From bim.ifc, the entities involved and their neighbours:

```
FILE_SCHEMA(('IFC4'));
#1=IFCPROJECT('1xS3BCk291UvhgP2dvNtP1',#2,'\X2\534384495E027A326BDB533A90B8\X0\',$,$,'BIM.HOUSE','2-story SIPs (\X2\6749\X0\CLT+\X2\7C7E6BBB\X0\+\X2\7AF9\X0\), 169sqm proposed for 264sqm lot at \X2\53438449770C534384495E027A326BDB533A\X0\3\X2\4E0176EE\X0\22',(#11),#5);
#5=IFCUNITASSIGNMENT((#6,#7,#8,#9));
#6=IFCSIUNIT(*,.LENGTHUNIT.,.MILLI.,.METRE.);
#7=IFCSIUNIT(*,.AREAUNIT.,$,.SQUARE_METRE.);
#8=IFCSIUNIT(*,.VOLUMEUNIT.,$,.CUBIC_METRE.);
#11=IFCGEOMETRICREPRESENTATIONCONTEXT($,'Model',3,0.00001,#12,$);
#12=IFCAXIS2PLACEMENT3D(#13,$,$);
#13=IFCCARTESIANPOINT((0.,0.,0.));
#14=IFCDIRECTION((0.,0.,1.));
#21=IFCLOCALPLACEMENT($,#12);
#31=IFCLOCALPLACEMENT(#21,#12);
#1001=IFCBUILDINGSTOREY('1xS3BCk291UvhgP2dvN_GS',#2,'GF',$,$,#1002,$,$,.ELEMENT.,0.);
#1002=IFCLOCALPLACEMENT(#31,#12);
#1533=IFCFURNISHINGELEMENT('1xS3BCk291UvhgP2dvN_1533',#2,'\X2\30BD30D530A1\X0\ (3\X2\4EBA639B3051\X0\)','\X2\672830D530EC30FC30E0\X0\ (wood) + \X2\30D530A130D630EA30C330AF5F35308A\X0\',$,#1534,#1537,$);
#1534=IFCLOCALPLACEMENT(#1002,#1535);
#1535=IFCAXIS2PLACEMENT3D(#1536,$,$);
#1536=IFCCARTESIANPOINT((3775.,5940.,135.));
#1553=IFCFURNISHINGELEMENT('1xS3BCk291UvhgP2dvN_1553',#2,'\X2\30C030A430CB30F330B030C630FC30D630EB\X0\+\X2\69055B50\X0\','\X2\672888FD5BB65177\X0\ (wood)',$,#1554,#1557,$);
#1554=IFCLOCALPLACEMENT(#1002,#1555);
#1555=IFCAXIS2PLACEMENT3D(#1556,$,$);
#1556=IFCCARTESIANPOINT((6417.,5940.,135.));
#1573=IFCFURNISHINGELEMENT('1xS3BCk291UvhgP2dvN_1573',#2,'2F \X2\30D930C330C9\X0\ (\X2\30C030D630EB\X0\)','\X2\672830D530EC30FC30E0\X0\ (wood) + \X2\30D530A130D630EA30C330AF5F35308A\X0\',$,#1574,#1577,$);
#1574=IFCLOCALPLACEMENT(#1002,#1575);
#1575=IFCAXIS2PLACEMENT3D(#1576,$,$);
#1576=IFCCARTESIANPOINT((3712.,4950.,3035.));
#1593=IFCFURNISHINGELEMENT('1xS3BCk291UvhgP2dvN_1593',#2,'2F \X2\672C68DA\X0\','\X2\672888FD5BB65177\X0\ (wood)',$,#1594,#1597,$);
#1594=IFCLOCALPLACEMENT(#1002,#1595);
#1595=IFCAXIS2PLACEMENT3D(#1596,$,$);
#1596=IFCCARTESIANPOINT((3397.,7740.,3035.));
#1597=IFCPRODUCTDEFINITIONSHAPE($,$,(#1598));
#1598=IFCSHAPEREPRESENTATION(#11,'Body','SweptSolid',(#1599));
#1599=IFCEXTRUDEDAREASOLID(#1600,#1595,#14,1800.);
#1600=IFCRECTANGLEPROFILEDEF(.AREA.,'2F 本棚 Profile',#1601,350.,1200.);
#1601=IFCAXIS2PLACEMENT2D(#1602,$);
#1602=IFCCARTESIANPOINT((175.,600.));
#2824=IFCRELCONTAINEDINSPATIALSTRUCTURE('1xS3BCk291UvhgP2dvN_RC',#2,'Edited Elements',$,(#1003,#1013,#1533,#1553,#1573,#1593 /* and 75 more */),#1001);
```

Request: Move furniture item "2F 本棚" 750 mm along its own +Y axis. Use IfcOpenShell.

```python
import ifcopenshell
import ifcopenshell.api.geometry
import ifcopenshell.util.placement
import ifcopenshell.util.unit

model = ifcopenshell.open("bim.ifc")
unit_scale = ifcopenshell.util.unit.calculate_unit_scale(model)

item = model.by_id(1593)
matrix = ifcopenshell.util.placement.get_local_placement(item.ObjectPlacement)
matrix[:3, 3] += matrix[:3, 1] * 0.75 / unit_scale
ifcopenshell.api.geometry.edit_object_placement(model, product=item, matrix=matrix, is_si=False)

print(ifcopenshell.util.placement.get_local_placement(item.ObjectPlacement).round(3) + 0.0)

model.write("bim_edited.ifc")
```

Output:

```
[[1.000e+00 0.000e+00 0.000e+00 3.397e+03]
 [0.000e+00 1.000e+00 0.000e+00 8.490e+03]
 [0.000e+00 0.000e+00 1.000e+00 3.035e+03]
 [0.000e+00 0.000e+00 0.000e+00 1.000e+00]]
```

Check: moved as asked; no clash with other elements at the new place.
